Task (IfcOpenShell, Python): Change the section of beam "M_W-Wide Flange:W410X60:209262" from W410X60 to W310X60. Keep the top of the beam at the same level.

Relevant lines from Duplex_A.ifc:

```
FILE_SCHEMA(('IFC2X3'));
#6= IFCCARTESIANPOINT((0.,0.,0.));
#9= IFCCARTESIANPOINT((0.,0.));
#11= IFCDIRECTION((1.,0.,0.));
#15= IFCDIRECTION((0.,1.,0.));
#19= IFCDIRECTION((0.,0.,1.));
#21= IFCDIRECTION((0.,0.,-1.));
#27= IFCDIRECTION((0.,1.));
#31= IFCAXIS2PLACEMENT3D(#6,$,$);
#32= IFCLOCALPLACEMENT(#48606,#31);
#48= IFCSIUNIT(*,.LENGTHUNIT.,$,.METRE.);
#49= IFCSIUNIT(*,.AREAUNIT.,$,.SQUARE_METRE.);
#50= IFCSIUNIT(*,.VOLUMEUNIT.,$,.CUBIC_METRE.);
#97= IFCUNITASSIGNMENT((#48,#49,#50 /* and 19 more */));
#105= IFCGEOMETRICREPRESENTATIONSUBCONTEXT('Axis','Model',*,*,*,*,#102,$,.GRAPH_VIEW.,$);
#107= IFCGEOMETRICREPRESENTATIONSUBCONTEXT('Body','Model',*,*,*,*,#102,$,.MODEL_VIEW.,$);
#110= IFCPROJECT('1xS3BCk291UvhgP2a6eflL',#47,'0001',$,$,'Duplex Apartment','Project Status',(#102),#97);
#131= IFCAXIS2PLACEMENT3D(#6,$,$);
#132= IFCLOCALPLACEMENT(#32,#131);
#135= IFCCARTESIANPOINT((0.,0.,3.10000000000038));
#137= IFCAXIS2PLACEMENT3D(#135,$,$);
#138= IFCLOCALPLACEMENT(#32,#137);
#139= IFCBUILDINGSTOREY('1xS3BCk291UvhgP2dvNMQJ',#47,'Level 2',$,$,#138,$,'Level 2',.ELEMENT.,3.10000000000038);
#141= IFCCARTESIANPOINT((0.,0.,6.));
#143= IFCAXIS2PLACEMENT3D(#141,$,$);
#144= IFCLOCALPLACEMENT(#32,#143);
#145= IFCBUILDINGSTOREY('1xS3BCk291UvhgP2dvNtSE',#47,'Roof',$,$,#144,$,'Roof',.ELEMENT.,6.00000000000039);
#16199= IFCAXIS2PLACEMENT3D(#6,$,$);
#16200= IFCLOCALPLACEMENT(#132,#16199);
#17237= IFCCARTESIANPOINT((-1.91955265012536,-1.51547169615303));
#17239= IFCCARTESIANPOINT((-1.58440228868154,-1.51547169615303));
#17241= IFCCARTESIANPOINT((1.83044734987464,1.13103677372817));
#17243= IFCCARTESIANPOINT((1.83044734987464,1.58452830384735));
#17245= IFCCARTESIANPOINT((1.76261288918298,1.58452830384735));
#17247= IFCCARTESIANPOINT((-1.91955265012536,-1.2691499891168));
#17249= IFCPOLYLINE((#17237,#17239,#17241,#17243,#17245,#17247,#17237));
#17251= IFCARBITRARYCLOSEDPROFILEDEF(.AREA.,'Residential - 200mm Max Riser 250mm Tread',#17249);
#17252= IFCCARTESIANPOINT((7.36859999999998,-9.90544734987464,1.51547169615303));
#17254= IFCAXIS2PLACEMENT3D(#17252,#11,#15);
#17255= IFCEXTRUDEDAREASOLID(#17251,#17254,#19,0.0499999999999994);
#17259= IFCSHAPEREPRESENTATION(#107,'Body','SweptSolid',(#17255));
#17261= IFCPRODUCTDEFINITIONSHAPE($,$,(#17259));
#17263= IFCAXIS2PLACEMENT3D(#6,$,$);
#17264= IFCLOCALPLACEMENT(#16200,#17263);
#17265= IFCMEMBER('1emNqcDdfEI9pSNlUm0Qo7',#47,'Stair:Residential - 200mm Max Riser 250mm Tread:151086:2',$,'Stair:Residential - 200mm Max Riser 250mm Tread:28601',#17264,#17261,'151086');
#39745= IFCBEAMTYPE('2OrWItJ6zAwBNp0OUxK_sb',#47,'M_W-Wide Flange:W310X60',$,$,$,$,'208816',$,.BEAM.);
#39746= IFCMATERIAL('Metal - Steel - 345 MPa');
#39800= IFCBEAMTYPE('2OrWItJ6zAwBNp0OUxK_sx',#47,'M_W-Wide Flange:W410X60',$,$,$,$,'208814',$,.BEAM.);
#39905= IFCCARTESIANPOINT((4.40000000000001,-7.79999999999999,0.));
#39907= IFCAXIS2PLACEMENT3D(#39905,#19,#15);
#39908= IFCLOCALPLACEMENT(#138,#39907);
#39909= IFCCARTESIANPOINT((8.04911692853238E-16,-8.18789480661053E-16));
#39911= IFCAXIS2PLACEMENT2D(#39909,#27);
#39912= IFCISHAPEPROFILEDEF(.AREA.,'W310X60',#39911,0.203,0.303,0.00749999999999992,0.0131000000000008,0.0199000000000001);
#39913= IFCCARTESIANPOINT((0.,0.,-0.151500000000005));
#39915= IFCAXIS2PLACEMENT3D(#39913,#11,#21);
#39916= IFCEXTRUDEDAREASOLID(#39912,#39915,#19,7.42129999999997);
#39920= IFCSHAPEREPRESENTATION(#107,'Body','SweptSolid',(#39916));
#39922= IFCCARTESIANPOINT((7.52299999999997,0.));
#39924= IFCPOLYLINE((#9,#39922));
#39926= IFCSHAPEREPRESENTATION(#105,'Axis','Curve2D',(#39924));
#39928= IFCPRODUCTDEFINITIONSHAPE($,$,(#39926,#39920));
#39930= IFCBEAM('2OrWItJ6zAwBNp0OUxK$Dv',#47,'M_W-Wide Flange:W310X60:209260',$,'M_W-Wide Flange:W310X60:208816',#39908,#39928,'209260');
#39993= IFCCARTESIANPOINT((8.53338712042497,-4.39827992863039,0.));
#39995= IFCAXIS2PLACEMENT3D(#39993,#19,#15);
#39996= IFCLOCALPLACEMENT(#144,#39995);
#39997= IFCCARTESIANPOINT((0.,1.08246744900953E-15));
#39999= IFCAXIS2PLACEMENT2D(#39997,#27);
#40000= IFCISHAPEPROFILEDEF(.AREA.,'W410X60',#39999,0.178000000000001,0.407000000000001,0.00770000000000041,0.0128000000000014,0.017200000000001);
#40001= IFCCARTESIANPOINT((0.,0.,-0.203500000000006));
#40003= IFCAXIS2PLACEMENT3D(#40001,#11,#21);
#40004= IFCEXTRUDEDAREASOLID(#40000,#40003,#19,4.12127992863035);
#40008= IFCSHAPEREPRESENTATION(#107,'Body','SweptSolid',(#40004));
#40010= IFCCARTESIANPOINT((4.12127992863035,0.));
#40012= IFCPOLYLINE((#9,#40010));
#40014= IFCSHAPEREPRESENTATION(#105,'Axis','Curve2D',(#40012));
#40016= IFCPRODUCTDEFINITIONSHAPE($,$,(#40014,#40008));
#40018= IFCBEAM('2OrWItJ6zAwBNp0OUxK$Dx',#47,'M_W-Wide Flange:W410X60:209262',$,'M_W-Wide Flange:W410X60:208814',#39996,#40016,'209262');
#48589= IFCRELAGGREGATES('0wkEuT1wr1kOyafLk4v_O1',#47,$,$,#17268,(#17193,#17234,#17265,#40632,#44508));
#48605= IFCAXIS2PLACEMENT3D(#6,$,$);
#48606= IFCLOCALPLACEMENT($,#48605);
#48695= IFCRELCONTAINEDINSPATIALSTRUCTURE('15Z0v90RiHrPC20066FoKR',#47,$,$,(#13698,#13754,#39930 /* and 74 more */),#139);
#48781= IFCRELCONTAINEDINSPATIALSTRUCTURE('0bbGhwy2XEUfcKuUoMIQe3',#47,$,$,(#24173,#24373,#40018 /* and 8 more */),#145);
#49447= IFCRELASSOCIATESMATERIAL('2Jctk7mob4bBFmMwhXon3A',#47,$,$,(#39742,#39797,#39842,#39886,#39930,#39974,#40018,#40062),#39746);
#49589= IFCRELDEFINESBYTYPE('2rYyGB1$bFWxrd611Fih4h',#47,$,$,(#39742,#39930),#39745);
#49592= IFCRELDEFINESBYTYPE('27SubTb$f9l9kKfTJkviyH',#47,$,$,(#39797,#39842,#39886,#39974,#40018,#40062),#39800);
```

```python
import ifcopenshell
import ifcopenshell.api.type
import ifcopenshell.util.element
import ifcopenshell.util.representation

model = ifcopenshell.open("Duplex_A.ifc")

member = model.by_guid("2OrWItJ6zAwBNp0OUxK$Dx")
source = next(p for p in model.by_type("IfcIShapeProfileDef") if p.ProfileName == "W310X60")

body = ifcopenshell.util.representation.get_representation(member, "Model", "Body")
solid = body.Items[0]
old_profile = solid.SweptArea

# Copy the section's sizes but keep this member's own profile position.
profile = ifcopenshell.util.element.copy(model, source)
# Profiles are centred, so shift by half the change in depth to hold the top.
shift = (old_profile.OverallDepth - profile.OverallDepth) / 2
x, y = old_profile.Position.Location.Coordinates
up = (-1.0, 0.0)  # upwards, in the solid's own plane
location = model.createIfcCartesianPoint((x + up[0] * shift, y + up[1] * shift))
profile.Position = model.createIfcAxis2Placement2D(location, old_profile.Position.RefDirection)
solid.SweptArea = profile
if not model.get_total_inverses(old_profile):
    ifcopenshell.util.element.remove_deep2(model, old_profile)

new_type = model.by_guid("2OrWItJ6zAwBNp0OUxK_sb")
ifcopenshell.api.type.assign_type(
    model, related_objects=[member], relating_type=new_type, should_map_representations=False
)
member.Name = member.Name.replace("W410X60", "W310X60")
member.ObjectType = "M_W-Wide Flange:W310X60:208814"

print(solid.SweptArea)

model.write("Duplex_A-out.ifc")
```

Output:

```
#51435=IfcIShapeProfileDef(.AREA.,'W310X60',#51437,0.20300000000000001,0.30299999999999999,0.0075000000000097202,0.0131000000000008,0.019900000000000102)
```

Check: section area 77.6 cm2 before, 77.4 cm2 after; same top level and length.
